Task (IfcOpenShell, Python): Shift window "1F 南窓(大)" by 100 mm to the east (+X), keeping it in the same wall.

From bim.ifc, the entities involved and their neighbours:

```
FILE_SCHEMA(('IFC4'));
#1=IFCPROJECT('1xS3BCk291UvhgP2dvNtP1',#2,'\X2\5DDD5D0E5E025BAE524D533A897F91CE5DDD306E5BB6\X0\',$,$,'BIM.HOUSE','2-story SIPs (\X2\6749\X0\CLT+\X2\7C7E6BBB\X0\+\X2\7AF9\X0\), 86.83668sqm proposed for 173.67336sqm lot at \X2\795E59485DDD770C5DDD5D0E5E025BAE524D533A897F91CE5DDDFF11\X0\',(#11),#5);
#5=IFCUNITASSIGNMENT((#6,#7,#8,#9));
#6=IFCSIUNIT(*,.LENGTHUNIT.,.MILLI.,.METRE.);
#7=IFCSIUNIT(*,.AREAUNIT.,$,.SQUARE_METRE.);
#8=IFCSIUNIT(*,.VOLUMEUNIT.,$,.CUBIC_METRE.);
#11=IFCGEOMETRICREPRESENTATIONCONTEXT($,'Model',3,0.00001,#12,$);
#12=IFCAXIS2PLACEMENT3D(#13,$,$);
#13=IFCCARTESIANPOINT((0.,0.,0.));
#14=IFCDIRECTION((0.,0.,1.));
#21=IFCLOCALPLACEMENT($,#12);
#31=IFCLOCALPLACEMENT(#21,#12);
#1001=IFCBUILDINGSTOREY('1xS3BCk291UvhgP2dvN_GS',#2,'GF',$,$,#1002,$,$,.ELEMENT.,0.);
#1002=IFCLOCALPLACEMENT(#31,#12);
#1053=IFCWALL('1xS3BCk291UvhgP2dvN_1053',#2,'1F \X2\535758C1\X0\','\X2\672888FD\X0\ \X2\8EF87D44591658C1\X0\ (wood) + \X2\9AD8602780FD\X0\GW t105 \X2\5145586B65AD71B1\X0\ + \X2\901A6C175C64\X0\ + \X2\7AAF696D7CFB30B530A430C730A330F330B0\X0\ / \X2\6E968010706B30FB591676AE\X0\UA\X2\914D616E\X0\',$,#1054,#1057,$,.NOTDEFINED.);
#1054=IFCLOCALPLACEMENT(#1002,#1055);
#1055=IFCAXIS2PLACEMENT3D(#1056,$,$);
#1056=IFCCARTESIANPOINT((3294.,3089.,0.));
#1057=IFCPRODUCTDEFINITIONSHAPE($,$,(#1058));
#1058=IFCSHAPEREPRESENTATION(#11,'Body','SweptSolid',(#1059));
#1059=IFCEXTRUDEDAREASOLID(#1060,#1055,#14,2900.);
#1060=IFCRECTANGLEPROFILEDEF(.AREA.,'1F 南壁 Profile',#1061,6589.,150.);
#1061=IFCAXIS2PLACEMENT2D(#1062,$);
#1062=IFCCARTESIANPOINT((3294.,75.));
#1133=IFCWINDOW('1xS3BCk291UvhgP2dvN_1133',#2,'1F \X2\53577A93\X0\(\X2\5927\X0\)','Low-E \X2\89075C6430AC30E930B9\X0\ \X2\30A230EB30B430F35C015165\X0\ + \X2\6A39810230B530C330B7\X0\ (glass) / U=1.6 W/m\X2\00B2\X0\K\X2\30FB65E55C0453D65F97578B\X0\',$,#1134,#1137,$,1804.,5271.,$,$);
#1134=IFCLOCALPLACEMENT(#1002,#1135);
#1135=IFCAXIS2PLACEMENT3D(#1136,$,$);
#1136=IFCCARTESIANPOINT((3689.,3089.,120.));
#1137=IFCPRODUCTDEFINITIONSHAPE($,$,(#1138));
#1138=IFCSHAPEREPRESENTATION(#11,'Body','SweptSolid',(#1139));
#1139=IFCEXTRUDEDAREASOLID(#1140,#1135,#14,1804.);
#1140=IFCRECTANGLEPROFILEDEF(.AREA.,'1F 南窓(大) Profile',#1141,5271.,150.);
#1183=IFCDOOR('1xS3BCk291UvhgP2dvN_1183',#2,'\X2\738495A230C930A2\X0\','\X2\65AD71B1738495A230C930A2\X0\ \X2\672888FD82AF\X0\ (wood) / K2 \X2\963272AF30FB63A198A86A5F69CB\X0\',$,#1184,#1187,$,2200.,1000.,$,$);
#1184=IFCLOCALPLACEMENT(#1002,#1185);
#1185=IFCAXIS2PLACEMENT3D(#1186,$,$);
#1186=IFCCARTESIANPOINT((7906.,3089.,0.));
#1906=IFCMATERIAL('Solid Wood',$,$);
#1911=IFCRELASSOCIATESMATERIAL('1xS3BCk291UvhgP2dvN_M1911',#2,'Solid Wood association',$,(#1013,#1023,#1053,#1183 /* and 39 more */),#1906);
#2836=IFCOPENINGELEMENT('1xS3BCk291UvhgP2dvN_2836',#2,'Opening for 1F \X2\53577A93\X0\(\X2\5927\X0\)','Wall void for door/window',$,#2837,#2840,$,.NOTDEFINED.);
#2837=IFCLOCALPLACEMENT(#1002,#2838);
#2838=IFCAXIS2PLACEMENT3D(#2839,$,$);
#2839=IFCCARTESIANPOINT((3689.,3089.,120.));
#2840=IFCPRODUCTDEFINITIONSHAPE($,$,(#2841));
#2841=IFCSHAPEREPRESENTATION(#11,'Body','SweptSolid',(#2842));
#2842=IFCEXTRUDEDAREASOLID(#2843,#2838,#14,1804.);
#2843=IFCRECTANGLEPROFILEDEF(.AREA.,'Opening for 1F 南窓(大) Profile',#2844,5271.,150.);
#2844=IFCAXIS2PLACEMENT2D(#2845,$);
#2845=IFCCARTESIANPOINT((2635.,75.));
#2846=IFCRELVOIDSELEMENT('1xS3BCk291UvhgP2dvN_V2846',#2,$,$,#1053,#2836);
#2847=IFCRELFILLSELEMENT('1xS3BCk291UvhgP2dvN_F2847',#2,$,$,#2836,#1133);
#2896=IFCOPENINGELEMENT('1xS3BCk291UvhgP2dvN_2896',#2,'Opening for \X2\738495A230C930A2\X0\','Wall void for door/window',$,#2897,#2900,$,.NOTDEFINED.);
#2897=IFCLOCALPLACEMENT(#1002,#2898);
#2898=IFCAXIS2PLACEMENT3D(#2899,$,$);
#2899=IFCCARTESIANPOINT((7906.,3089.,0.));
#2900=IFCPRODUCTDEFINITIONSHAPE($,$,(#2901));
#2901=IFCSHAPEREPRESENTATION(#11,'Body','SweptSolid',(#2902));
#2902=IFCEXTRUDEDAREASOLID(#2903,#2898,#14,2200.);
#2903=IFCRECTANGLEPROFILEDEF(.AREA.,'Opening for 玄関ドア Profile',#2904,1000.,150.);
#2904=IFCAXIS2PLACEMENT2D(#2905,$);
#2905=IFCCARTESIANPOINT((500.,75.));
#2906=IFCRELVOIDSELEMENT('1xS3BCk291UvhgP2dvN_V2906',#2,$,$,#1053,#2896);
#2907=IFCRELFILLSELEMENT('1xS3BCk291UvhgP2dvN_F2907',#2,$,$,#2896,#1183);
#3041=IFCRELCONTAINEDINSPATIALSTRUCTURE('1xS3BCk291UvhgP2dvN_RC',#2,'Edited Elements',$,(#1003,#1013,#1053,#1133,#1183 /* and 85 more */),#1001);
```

```python
import ifcopenshell
import ifcopenshell.api.geometry
import ifcopenshell.util.placement

model = ifcopenshell.open("bim.ifc")

window = model.by_guid("1xS3BCk291UvhgP2dvN_1133")
opening = window.FillsVoids[0].RelatingOpeningElement
wall = opening.VoidsElements[0].RelatingBuildingElement

wall_matrix = ifcopenshell.util.placement.get_local_placement(wall.ObjectPlacement)
shift = wall_matrix[:3, 0] * 100.0
before = ifcopenshell.util.placement.get_local_placement(window.ObjectPlacement)[:3, 3].copy()

# The window is not placed relative to its opening, so move both.
for product in (opening, window):
    matrix = ifcopenshell.util.placement.get_local_placement(product.ObjectPlacement)
    matrix[:3, 3] += shift
    ifcopenshell.api.geometry.edit_object_placement(model, product=product, matrix=matrix, is_si=False)

after = ifcopenshell.util.placement.get_local_placement(window.ObjectPlacement)[:3, 3]
print("window moved by", (after - before).round(3) + 0.0)

model.write("bim-out.ifc")
```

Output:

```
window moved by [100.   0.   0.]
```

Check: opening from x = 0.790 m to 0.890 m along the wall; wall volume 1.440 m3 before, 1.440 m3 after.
